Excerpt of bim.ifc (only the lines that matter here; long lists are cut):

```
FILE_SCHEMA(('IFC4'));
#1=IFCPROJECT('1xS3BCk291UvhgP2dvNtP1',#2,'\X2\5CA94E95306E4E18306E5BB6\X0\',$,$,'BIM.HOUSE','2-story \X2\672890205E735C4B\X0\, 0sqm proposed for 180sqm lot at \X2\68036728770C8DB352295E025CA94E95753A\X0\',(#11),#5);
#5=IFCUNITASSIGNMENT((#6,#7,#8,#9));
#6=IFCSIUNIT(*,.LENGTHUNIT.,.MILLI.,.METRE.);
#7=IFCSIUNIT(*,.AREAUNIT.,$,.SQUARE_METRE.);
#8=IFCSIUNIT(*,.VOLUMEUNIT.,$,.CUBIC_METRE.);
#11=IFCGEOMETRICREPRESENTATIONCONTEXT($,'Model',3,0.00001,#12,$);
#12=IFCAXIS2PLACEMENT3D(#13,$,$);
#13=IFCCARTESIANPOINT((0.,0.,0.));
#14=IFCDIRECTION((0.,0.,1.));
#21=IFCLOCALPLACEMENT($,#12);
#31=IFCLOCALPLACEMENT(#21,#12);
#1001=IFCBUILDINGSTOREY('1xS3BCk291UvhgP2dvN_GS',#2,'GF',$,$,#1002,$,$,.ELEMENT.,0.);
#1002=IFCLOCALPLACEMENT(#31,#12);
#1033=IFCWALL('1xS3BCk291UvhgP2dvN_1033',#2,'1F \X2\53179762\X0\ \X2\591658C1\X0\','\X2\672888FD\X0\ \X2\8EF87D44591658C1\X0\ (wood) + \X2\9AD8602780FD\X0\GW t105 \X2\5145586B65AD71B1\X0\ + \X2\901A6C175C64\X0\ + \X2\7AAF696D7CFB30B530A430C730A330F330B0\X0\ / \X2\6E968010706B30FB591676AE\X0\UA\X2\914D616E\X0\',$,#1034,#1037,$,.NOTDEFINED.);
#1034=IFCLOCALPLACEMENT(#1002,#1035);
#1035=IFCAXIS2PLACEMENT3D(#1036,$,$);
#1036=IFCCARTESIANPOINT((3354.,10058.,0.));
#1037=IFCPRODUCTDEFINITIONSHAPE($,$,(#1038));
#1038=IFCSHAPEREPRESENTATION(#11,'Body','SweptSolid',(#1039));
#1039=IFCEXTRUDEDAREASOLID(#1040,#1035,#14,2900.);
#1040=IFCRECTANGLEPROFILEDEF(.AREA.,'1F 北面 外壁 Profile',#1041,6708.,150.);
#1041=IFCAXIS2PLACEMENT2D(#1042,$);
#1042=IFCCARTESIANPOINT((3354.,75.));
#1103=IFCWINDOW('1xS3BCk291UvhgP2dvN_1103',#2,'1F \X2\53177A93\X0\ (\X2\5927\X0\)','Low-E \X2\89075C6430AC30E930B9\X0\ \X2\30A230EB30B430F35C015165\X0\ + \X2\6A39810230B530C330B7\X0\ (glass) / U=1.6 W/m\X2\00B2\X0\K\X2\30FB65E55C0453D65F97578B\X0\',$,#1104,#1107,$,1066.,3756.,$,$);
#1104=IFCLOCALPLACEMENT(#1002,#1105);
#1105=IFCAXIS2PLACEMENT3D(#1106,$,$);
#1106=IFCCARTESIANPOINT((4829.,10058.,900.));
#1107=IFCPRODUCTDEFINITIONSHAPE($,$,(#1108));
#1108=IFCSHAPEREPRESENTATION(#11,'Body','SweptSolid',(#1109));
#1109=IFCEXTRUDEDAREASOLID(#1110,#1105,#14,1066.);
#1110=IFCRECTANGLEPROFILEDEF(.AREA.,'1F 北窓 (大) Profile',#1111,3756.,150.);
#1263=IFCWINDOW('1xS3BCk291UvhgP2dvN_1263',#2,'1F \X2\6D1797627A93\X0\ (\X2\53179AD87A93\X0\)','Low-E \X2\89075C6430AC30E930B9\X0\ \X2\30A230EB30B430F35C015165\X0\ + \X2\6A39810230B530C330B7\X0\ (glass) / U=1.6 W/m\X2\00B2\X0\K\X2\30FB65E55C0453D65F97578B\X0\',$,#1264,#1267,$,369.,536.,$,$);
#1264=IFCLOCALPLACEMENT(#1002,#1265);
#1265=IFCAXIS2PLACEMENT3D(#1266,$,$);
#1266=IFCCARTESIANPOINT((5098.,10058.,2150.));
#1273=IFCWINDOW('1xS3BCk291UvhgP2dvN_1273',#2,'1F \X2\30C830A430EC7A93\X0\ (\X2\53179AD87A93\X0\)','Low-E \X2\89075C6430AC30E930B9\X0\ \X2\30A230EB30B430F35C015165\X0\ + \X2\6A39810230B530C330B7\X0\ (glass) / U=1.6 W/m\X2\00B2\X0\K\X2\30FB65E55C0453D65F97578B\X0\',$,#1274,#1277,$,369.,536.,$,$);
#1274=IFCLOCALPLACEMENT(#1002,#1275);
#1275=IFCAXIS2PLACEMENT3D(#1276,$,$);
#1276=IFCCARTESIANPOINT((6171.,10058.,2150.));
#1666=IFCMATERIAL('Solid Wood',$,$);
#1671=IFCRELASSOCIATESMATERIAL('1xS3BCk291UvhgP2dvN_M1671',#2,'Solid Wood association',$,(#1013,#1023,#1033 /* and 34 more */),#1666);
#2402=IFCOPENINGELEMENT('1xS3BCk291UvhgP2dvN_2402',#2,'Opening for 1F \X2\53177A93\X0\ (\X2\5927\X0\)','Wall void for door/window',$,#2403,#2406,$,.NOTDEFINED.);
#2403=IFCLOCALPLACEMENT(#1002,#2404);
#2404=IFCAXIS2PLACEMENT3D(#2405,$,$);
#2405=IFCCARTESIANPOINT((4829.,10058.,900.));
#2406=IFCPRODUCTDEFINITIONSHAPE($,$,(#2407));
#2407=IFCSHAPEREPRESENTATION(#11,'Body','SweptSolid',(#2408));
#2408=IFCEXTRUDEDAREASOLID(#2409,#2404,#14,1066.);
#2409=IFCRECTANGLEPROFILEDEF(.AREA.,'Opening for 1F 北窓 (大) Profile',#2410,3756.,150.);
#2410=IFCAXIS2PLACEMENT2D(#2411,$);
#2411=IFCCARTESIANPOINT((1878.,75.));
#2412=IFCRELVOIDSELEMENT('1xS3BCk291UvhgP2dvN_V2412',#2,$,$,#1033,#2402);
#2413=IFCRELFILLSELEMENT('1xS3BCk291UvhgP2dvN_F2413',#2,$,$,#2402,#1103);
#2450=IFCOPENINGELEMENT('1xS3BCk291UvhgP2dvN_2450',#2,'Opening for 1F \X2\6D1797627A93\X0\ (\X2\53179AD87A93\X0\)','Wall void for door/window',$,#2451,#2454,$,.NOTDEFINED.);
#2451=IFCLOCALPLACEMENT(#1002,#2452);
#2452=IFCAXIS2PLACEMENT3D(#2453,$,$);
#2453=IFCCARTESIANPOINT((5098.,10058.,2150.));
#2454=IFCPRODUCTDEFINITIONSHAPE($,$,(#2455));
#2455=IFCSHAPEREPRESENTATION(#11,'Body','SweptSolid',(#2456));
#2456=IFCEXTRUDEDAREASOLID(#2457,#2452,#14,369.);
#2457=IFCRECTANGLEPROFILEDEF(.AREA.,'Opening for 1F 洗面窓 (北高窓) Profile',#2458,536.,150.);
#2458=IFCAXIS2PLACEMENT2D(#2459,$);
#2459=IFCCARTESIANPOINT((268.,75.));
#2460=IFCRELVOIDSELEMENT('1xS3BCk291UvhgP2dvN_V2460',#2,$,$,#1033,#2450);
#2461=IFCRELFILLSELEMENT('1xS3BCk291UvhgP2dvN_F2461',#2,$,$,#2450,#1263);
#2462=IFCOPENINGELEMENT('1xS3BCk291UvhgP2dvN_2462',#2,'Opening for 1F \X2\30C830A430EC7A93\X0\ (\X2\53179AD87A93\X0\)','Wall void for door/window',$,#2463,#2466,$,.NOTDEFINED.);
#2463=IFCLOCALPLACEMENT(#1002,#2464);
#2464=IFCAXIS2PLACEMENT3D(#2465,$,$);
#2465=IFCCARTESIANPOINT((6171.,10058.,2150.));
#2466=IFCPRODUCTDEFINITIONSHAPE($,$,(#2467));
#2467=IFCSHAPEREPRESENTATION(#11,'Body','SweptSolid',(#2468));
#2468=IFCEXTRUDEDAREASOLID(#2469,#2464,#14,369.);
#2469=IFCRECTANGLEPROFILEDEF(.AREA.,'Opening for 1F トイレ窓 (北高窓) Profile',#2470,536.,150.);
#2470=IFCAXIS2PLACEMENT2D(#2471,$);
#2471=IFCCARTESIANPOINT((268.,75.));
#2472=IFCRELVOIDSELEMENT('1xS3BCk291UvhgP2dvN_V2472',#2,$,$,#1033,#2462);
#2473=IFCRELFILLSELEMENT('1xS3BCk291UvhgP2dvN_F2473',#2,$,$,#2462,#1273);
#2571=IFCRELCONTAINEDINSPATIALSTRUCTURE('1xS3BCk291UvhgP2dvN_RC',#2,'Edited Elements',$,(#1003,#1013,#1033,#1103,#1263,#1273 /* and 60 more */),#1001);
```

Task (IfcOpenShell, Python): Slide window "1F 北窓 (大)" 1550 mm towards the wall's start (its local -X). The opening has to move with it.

```python
import ifcopenshell
import ifcopenshell.api.geometry
import ifcopenshell.util.placement
import ifcopenshell.util.unit

model = ifcopenshell.open("bim.ifc")
unit_scale = ifcopenshell.util.unit.calculate_unit_scale(model)

window = model.by_guid("1xS3BCk291UvhgP2dvN_1103")
opening = window.FillsVoids[0].RelatingOpeningElement
wall = opening.VoidsElements[0].RelatingBuildingElement

wall_matrix = ifcopenshell.util.placement.get_local_placement(wall.ObjectPlacement)
shift = wall_matrix[:3, 0] * -1.55 / unit_scale
before = ifcopenshell.util.placement.get_local_placement(window.ObjectPlacement)[:3, 3].copy()

# The window is not placed relative to its opening, so move both.
for product in (opening, window):
    matrix = ifcopenshell.util.placement.get_local_placement(product.ObjectPlacement)
    matrix[:3, 3] += shift
    ifcopenshell.api.geometry.edit_object_placement(model, product=product, matrix=matrix, is_si=False)

after = ifcopenshell.util.placement.get_local_placement(window.ObjectPlacement)[:3, 3]
print("window moved by", (after - before).round(3) + 0.0)

model.write("bim_v2.ifc")
```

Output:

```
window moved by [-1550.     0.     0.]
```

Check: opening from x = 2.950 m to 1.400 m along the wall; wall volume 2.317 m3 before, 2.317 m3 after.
